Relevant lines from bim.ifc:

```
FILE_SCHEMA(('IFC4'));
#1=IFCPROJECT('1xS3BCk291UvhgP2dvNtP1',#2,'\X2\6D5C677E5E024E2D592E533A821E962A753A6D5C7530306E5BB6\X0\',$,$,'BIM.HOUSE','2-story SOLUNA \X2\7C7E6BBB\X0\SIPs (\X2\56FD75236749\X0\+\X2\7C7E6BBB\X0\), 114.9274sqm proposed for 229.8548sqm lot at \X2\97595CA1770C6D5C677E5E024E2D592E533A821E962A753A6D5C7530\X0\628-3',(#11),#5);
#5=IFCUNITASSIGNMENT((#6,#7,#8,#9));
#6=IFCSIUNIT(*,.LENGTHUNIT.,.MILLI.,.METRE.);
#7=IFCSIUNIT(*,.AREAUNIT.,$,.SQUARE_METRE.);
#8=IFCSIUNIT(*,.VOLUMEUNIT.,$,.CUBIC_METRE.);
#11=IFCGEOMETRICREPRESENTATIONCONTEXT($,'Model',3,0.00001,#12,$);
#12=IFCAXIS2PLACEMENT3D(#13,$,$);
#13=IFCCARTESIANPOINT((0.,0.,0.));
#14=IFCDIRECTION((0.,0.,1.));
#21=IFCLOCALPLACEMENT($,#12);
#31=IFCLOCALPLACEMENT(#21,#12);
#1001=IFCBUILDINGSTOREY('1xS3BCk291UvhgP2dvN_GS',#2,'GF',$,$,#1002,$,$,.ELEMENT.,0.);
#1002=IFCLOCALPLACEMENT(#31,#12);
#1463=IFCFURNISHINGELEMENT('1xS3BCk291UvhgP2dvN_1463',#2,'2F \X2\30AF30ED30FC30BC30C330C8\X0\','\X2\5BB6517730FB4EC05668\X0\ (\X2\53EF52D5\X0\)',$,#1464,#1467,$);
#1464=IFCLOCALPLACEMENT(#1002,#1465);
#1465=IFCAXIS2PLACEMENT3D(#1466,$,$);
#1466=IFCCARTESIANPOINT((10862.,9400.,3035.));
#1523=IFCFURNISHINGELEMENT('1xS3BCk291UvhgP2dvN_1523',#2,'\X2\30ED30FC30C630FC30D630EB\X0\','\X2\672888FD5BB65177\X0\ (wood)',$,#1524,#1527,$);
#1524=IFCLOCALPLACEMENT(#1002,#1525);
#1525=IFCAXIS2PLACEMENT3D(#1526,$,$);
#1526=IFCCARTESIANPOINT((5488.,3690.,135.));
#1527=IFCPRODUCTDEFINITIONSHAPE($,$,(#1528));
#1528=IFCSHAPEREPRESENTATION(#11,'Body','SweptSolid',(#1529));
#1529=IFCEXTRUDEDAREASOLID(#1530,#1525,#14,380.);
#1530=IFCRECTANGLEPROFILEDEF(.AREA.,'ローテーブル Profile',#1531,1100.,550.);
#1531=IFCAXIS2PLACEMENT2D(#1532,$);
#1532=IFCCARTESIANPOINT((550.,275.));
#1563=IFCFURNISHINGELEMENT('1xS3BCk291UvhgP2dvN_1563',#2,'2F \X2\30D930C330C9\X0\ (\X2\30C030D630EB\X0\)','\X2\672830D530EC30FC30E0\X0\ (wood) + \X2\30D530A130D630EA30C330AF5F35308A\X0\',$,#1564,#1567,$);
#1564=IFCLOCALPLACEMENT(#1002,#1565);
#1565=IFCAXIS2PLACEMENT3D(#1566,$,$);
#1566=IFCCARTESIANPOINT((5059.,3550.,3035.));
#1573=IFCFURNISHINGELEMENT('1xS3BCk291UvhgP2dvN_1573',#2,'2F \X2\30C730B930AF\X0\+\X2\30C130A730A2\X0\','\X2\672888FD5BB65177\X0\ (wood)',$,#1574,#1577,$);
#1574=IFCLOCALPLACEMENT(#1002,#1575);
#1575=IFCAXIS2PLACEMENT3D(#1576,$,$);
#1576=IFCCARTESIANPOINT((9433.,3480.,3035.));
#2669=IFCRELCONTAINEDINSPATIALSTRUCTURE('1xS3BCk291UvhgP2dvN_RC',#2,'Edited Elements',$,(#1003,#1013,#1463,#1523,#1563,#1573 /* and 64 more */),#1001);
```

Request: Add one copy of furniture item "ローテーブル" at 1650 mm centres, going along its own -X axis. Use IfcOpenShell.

```python
import ifcopenshell
import ifcopenshell.api.geometry
import ifcopenshell.api.root
import ifcopenshell.util.element
import ifcopenshell.util.placement
import ifcopenshell.util.unit

model = ifcopenshell.open("bim.ifc")
unit_scale = ifcopenshell.util.unit.calculate_unit_scale(model)


def reuse_history(source, copy):
    """copy_class also copies each property set's owner history, people and application; keep the originals."""
    for rel in copy.IsDefinedBy:
        if rel.is_a("IfcRelDefinesByProperties") and (history := rel.RelatingPropertyDefinition.OwnerHistory):
            rel.RelatingPropertyDefinition.OwnerHistory = source.OwnerHistory
            ifcopenshell.util.element.remove_deep2(model, history)


source = model.by_guid("1xS3BCk291UvhgP2dvN_1523")
base = ifcopenshell.util.placement.get_local_placement(source.ObjectPlacement)
step = -base[:3, 0] * 1.65 / unit_scale

for i in range(1, 2):
    copy = ifcopenshell.api.root.copy_class(model, product=source)
    copy.Representation = ifcopenshell.util.element.copy_deep(
        model, source.Representation, exclude=["IfcGeometricRepresentationContext", "IfcRepresentationMap"]
    )
    reuse_history(source, copy)
    matrix = base.copy()
    matrix[:3, 3] += i * step
    print("added at", matrix[:3, 3].round(3) + 0.0)
    ifcopenshell.api.geometry.edit_object_placement(model, product=copy, matrix=matrix, is_si=False)

model.write("bim_edited.ifc")
```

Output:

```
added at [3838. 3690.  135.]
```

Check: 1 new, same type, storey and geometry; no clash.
